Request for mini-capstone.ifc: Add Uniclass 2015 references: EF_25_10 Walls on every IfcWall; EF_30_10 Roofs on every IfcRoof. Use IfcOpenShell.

First a look at what the model holds.

```python
import ifcopenshell

model = ifcopenshell.open("mini-capstone.ifc")
print(model.schema)
print("classifications:", [c.Name for c in model.by_type("IfcClassification")])
for ifc_class in ("IfcDoor", "IfcRoof", "IfcStair", "IfcWall", "IfcWindow"):
    print(ifc_class, len(model.by_type(ifc_class)))
```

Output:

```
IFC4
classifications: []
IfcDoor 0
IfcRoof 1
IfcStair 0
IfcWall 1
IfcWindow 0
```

```python
import ifcopenshell
import ifcopenshell.api.classification

model = ifcopenshell.open("mini-capstone.ifc")

system = ifcopenshell.api.classification.add_classification(model, classification="Uniclass 2015")

codes = {
    "IfcWall": ("EF_25_10", "Walls"),
    "IfcRoof": ("EF_30_10", "Roofs"),
}
for ifc_class, (code, name) in codes.items():
    products = model.by_type(ifc_class)
    ifcopenshell.api.classification.add_reference(
        model, products=products, classification=system, identification=code, name=name
    )
    print(code, len(products))

model.write("mini-capstone-out.ifc")
```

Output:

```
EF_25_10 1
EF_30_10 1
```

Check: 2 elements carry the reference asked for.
